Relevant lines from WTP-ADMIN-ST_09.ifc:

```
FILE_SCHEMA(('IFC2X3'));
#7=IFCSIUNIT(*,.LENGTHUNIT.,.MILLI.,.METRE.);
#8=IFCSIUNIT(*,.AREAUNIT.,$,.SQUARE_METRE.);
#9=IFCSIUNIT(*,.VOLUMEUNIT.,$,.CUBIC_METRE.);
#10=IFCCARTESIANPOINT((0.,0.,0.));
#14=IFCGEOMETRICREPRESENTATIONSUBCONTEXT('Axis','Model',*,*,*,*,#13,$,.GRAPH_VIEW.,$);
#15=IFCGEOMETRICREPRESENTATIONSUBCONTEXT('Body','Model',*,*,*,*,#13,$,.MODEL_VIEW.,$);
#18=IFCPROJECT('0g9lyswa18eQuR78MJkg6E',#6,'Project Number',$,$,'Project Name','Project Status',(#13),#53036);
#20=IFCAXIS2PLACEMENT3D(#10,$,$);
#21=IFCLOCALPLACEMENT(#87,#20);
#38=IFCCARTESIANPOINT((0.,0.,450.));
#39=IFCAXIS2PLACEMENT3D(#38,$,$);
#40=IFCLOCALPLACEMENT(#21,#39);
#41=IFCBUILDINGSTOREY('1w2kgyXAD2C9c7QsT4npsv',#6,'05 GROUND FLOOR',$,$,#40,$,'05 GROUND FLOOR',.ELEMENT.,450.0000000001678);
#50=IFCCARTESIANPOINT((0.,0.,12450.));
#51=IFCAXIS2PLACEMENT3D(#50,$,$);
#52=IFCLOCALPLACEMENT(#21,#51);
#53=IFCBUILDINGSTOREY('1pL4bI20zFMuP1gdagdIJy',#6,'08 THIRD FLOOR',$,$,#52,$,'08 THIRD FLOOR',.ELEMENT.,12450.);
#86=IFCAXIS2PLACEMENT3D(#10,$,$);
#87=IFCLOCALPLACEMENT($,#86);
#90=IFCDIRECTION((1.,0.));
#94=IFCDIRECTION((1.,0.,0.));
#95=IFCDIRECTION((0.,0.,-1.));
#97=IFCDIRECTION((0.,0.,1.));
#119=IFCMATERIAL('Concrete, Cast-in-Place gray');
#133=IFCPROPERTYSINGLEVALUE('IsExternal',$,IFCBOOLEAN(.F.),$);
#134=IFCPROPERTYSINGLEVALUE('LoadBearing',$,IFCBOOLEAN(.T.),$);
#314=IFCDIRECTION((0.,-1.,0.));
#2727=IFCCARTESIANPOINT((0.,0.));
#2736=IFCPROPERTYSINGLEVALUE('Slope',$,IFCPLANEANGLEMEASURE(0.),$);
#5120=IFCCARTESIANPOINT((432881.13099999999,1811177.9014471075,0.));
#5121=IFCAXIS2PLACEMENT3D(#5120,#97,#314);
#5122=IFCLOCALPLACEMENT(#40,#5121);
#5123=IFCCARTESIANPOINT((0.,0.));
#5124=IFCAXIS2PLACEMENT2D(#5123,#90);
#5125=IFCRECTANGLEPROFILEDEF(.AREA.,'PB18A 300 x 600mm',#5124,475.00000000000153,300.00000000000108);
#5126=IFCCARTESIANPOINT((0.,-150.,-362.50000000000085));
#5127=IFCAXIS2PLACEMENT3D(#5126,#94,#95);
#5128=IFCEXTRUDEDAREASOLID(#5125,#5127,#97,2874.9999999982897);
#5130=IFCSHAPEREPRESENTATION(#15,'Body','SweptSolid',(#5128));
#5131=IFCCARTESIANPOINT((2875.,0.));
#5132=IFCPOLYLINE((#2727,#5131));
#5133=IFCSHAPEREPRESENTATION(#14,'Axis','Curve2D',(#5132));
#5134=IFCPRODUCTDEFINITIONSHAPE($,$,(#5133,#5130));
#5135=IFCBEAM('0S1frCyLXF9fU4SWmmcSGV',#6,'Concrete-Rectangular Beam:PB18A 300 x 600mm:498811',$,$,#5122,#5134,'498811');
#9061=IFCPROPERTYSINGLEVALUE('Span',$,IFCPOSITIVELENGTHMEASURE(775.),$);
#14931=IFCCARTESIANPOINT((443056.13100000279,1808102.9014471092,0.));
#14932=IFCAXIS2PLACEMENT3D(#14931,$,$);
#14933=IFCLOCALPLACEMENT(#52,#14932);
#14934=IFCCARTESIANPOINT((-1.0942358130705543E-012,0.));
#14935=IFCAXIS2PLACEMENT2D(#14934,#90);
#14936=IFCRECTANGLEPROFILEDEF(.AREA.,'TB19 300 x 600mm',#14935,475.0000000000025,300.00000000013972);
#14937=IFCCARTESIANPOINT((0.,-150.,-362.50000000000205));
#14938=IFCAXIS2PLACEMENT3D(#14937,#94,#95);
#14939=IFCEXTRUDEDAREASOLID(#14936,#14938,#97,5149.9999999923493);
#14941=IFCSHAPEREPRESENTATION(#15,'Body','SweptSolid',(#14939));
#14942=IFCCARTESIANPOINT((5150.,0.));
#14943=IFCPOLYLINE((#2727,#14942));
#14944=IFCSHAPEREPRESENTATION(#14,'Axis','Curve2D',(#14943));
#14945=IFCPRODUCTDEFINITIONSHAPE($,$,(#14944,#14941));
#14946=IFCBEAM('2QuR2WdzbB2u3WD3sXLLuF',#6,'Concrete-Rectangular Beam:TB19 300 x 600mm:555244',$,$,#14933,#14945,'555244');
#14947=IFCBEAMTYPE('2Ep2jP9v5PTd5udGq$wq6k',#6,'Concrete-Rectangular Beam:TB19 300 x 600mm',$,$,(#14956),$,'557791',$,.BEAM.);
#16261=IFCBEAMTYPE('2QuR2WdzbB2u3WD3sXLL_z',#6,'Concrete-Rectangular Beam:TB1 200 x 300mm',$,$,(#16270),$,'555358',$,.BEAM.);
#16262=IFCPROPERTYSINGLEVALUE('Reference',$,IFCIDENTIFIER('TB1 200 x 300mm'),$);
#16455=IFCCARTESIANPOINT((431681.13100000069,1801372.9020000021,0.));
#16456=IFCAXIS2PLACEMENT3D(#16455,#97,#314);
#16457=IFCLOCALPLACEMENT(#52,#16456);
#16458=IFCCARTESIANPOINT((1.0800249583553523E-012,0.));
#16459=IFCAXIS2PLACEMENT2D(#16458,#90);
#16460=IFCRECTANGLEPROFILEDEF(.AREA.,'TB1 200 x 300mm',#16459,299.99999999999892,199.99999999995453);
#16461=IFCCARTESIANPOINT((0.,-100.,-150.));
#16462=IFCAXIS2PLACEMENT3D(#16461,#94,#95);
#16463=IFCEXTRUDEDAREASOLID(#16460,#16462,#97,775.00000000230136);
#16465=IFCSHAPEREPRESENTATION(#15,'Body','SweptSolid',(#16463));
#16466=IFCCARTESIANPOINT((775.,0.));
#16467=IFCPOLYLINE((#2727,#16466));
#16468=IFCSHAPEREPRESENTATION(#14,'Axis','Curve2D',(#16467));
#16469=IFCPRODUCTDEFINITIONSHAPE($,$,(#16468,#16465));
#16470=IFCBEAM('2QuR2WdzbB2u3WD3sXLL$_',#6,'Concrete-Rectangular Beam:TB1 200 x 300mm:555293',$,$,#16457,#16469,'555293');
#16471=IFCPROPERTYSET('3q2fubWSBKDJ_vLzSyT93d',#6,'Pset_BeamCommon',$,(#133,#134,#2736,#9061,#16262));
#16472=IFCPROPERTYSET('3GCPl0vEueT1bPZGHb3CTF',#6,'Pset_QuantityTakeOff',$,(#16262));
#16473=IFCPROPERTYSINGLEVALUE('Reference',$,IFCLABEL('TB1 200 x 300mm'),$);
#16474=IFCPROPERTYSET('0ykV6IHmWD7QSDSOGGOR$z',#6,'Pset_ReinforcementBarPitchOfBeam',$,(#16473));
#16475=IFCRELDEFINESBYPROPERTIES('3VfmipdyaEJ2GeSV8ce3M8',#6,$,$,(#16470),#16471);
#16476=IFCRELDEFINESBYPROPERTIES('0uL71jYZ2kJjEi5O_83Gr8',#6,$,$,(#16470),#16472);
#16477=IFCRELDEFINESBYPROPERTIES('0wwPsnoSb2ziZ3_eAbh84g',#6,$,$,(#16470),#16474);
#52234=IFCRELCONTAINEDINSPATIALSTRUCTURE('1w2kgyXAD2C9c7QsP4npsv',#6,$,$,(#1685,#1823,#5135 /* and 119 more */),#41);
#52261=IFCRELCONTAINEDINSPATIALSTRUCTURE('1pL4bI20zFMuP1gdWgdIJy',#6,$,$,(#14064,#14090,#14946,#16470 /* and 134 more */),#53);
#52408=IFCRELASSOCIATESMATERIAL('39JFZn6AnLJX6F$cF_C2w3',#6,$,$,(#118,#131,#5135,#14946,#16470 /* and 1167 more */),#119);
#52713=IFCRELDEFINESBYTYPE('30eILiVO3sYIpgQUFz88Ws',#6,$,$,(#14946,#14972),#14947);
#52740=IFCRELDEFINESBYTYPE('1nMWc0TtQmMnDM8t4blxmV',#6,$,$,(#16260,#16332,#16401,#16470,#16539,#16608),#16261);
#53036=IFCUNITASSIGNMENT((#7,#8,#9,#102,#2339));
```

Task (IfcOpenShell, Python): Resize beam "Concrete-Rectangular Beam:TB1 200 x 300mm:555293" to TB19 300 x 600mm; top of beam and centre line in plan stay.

```python
import ifcopenshell
import ifcopenshell.api.pset
import ifcopenshell.api.type
import ifcopenshell.util.element
import ifcopenshell.util.representation

model = ifcopenshell.open("WTP-ADMIN-ST_09.ifc")

member = model.by_id(16470)
source = next(p for p in model.by_type("IfcRectangleProfileDef") if p.ProfileName == "TB19 300 x 600mm")

body = ifcopenshell.util.representation.get_representation(member, "Model", "Body")
solid = body.Items[0]
old_profile = solid.SweptArea

# Copy the section's sizes but keep this member's own profile position.
profile = ifcopenshell.util.element.copy(model, source)
# Profiles are centred, so shift by half the change in depth to hold the top.
shift = (old_profile.XDim - profile.XDim) / 2
x, y = old_profile.Position.Location.Coordinates
up = (-1.0, 0.0)  # upwards, in the solid's own plane
location = model.createIfcCartesianPoint((x + up[0] * shift, y + up[1] * shift))
profile.Position = model.createIfcAxis2Placement2D(location, old_profile.Position.RefDirection)
solid.SweptArea = profile
if not model.get_total_inverses(old_profile):
    ifcopenshell.util.element.remove_deep2(model, old_profile)

new_type = model.by_guid("2Ep2jP9v5PTd5udGq$wq6k")
ifcopenshell.api.type.assign_type(
    model, related_objects=[member], relating_type=new_type, should_map_representations=False
)
member.Name = member.Name.replace("TB1 200 x 300mm", "TB19 300 x 600mm")
pset = model.by_id(ifcopenshell.util.element.get_pset(member, "Pset_BeamCommon", should_inherit=False)["id"])
ifcopenshell.api.pset.edit_pset(model, pset=pset, properties={"Reference": "TB19 300 x 600mm"})
pset = model.by_id(ifcopenshell.util.element.get_pset(member, "Pset_QuantityTakeOff", should_inherit=False)["id"])
ifcopenshell.api.pset.edit_pset(model, pset=pset, properties={"Reference": "TB19 300 x 600mm"})
pset = model.by_id(ifcopenshell.util.element.get_pset(member, "Pset_ReinforcementBarPitchOfBeam", should_inherit=False)["id"])
ifcopenshell.api.pset.edit_pset(model, pset=pset, properties={"Reference": "TB19 300 x 600mm"})

print(solid.SweptArea)

model.write("WTP-ADMIN-ST_09_rev.ifc")
```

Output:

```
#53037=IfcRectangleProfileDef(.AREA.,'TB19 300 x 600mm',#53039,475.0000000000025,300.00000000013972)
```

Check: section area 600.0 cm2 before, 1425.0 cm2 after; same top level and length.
